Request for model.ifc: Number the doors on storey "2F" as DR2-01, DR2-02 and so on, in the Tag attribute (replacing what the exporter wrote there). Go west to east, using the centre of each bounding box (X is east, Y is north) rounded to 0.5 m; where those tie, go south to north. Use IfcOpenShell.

First a look at what the model holds.

```python
import ifcopenshell
import ifcopenshell.util.element
import ifcopenshell.util.placement

model = ifcopenshell.open("model.ifc")
print(model.schema)
storey = next(s for s in model.by_type("IfcBuildingStorey") if s.Name == "2F")
doors = [e for e in ifcopenshell.util.element.get_decomposition(storey) if e.is_a("IfcDoor")]
for e in sorted(doors, key=lambda e: e.id()):
    origin = ifcopenshell.util.placement.get_local_placement(e.ObjectPlacement)[:3, 3]
    print(e.id(), e.Tag, e.Name, origin.round(2) + 0.0, sep=" | ")
```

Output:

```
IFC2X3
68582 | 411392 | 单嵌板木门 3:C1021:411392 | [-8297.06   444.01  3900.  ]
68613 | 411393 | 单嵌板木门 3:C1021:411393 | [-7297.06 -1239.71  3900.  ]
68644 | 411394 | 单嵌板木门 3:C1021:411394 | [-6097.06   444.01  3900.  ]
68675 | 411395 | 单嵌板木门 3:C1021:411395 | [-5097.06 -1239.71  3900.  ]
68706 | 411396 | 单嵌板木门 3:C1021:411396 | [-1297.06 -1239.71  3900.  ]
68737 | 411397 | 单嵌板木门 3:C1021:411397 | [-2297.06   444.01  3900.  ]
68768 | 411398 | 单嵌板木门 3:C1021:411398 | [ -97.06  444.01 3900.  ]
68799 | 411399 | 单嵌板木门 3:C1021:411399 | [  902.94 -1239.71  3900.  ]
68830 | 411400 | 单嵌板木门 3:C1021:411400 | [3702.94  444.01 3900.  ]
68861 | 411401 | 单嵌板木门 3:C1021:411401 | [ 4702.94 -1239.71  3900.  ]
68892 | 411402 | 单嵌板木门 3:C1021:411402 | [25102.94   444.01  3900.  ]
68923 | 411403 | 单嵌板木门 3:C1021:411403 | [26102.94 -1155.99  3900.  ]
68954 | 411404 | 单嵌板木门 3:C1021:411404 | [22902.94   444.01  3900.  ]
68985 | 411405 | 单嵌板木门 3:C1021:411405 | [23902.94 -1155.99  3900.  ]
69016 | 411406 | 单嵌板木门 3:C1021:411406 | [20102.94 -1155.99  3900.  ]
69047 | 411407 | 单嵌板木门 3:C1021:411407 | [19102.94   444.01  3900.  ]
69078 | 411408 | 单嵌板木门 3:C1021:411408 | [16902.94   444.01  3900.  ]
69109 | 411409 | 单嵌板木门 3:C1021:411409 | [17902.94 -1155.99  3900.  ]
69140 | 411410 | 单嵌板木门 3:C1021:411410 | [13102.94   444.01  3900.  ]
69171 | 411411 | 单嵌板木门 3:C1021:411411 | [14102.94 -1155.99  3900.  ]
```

```python
import ifcopenshell
import ifcopenshell.geom
import ifcopenshell.util.element
import ifcopenshell.util.shape

model = ifcopenshell.open("model.ifc")
settings = ifcopenshell.geom.settings()
settings.set("use-world-coords", True)


def centre(element):
    shape = ifcopenshell.geom.create_shape(settings, element)
    return ifcopenshell.util.shape.get_bbox_centroid(shape.geometry)


storey = next(s for s in model.by_type("IfcBuildingStorey") if s.Name == "2F")
doors = [e for e in ifcopenshell.util.element.get_decomposition(storey) if e.is_a("IfcDoor")]

# Insertion points can sit at a corner or the storey origin, so sort by the geometry (in metres).
centres = {e: centre(e) for e in doors}
doors.sort(key=lambda e: (round(centres[e][0] / 0.5), centres[e][1]))

for i, e in enumerate(doors, start=1):
    number = f"DR2-{i:02d}"
    e.Tag = number
    print(e.id(), number)

model.write("model_updated.ifc")
```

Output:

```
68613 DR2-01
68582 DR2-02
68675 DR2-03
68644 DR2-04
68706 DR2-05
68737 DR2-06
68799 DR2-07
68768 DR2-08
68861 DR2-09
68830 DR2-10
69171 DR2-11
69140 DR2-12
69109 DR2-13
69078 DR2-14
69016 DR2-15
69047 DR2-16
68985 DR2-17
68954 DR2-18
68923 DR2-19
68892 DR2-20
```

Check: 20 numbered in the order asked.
